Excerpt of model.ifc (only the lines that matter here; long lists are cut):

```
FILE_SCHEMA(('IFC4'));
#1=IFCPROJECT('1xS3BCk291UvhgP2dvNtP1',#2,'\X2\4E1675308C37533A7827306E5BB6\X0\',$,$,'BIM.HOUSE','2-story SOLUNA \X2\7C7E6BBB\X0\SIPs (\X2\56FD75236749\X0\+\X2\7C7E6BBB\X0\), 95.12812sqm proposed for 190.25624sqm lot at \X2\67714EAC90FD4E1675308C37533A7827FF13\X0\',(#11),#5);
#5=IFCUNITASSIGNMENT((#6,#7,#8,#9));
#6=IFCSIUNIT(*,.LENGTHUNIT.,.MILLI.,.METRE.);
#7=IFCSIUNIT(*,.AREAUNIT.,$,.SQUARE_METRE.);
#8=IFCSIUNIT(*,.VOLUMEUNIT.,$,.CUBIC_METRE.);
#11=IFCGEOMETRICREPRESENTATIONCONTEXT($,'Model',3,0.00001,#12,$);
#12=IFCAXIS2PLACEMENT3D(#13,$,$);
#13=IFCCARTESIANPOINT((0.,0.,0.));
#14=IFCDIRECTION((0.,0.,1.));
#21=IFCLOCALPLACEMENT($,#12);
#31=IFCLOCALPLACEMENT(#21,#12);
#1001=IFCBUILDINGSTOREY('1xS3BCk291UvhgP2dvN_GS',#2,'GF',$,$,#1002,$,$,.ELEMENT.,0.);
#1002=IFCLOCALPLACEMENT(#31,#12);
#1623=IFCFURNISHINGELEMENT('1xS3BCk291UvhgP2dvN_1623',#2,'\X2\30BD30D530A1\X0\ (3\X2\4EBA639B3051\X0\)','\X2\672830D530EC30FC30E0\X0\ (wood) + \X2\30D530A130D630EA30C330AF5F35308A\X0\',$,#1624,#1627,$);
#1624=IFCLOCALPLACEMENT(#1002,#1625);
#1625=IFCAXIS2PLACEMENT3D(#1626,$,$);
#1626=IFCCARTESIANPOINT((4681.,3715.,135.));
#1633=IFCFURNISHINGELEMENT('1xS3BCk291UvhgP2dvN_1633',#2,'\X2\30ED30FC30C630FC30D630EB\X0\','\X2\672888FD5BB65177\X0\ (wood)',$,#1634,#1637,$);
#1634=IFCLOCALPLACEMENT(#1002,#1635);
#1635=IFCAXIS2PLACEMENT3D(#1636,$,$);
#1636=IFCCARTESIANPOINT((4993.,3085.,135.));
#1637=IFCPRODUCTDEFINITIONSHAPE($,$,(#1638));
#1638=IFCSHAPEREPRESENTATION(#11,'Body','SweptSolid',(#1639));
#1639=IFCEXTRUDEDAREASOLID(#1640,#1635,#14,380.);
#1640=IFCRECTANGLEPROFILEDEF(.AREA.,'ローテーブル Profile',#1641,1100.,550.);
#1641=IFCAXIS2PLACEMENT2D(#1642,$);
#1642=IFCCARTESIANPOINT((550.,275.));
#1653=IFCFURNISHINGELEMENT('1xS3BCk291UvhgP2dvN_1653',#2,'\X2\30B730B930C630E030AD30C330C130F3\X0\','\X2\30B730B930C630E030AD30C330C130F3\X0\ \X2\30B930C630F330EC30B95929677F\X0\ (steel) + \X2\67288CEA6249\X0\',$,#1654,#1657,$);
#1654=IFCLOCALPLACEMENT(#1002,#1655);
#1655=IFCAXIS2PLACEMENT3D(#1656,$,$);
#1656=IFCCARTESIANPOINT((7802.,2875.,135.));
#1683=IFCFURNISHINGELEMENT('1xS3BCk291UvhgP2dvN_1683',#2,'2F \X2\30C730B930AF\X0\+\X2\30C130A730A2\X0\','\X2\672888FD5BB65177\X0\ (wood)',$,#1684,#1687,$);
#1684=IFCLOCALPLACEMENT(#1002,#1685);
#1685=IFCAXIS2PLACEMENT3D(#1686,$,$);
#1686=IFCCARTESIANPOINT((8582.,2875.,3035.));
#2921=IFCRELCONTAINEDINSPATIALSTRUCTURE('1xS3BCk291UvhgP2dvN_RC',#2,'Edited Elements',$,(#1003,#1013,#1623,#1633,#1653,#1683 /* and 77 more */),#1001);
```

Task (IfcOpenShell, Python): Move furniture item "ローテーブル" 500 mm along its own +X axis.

```python
import ifcopenshell
import ifcopenshell.api.geometry
import ifcopenshell.util.placement
import ifcopenshell.util.unit

model = ifcopenshell.open("model.ifc")
unit_scale = ifcopenshell.util.unit.calculate_unit_scale(model)

item = model.by_guid("1xS3BCk291UvhgP2dvN_1633")
matrix = ifcopenshell.util.placement.get_local_placement(item.ObjectPlacement)
matrix[:3, 3] += matrix[:3, 0] * 0.5 / unit_scale
ifcopenshell.api.geometry.edit_object_placement(model, product=item, matrix=matrix, is_si=False)

print(ifcopenshell.util.placement.get_local_placement(item.ObjectPlacement).round(3) + 0.0)

model.write("model_updated.ifc")
```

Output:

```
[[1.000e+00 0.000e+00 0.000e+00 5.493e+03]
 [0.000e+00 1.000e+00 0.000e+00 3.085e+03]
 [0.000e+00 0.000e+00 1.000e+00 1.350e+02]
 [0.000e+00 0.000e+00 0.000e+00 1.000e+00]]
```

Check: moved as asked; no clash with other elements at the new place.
